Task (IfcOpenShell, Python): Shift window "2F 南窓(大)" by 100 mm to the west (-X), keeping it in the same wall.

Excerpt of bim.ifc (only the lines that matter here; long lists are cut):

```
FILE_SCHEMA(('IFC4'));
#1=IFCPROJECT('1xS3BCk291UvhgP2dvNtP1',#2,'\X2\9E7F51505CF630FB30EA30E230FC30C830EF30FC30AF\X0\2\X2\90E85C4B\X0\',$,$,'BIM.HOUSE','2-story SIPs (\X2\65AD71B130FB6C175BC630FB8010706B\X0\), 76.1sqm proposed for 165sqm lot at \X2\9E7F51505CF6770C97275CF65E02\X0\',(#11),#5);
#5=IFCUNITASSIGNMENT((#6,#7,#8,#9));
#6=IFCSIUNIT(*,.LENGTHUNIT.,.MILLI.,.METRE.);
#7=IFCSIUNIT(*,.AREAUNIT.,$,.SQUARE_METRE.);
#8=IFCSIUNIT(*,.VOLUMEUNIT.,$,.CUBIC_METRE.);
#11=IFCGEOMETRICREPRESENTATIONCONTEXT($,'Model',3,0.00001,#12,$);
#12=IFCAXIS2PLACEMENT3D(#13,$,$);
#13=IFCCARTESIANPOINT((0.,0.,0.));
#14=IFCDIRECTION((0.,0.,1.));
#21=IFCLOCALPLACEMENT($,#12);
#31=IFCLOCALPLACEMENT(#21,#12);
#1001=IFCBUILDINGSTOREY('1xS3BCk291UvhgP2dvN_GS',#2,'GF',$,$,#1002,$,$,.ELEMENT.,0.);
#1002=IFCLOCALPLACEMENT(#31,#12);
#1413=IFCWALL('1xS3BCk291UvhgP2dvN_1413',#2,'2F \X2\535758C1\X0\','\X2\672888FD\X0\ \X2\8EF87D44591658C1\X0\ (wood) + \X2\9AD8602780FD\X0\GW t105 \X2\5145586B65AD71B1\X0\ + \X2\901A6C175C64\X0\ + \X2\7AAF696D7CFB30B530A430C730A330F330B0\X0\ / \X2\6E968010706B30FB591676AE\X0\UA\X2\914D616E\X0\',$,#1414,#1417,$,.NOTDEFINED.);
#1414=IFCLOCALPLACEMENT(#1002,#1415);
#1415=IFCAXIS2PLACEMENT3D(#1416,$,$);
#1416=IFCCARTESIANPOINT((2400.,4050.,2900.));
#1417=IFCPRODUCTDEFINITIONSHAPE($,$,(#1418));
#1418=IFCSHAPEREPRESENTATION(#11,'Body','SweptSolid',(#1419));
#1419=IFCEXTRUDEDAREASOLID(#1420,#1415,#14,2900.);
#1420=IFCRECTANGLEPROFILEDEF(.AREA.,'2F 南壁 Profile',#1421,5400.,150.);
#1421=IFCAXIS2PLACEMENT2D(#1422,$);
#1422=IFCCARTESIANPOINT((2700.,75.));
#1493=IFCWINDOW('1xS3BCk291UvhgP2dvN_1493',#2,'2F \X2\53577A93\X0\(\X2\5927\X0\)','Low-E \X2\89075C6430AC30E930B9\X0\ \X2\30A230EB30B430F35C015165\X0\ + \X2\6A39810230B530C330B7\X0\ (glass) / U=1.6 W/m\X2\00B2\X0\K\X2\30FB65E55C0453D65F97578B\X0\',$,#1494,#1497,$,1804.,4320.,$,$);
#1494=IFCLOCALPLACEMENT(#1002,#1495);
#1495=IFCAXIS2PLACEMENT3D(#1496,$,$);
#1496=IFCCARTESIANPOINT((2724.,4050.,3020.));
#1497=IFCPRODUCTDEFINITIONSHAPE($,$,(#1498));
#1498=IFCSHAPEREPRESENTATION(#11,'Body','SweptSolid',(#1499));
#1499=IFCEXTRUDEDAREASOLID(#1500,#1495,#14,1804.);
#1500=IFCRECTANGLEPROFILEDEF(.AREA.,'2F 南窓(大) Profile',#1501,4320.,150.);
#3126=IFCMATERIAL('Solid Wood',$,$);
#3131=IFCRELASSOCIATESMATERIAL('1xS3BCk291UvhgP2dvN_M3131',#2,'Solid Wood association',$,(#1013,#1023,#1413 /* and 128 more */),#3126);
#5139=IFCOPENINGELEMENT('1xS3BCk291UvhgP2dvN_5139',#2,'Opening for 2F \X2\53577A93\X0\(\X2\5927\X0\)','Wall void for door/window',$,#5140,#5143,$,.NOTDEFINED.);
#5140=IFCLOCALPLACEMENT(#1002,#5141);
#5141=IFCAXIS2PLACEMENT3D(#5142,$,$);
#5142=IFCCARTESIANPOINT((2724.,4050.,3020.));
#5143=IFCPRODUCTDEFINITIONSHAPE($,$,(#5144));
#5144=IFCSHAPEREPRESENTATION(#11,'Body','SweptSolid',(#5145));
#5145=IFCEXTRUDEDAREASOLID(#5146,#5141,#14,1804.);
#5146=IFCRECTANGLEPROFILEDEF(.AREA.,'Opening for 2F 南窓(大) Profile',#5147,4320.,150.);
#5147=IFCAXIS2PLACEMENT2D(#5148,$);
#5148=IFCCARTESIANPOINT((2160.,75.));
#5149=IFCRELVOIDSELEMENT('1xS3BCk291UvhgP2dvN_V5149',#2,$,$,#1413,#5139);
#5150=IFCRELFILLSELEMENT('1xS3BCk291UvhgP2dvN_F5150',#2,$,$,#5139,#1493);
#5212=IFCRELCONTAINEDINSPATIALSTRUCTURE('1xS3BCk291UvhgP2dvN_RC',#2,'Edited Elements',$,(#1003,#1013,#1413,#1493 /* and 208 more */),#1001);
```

```python
import ifcopenshell
import ifcopenshell.api.geometry
import ifcopenshell.util.placement

model = ifcopenshell.open("bim.ifc")

window = model.by_id(1493)
opening = window.FillsVoids[0].RelatingOpeningElement
wall = opening.VoidsElements[0].RelatingBuildingElement

wall_matrix = ifcopenshell.util.placement.get_local_placement(wall.ObjectPlacement)
shift = wall_matrix[:3, 0] * -100.0
before = ifcopenshell.util.placement.get_local_placement(window.ObjectPlacement)[:3, 3].copy()

# The window is not placed relative to its opening, so move both.
for product in (opening, window):
    matrix = ifcopenshell.util.placement.get_local_placement(product.ObjectPlacement)
    matrix[:3, 3] += shift
    ifcopenshell.api.geometry.edit_object_placement(model, product=product, matrix=matrix, is_si=False)

after = ifcopenshell.util.placement.get_local_placement(window.ObjectPlacement)[:3, 3]
print("window moved by", (after - before).round(3) + 0.0)

model.write("bim_v2.ifc")
```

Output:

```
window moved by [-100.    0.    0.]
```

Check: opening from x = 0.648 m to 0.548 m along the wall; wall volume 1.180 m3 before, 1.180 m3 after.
